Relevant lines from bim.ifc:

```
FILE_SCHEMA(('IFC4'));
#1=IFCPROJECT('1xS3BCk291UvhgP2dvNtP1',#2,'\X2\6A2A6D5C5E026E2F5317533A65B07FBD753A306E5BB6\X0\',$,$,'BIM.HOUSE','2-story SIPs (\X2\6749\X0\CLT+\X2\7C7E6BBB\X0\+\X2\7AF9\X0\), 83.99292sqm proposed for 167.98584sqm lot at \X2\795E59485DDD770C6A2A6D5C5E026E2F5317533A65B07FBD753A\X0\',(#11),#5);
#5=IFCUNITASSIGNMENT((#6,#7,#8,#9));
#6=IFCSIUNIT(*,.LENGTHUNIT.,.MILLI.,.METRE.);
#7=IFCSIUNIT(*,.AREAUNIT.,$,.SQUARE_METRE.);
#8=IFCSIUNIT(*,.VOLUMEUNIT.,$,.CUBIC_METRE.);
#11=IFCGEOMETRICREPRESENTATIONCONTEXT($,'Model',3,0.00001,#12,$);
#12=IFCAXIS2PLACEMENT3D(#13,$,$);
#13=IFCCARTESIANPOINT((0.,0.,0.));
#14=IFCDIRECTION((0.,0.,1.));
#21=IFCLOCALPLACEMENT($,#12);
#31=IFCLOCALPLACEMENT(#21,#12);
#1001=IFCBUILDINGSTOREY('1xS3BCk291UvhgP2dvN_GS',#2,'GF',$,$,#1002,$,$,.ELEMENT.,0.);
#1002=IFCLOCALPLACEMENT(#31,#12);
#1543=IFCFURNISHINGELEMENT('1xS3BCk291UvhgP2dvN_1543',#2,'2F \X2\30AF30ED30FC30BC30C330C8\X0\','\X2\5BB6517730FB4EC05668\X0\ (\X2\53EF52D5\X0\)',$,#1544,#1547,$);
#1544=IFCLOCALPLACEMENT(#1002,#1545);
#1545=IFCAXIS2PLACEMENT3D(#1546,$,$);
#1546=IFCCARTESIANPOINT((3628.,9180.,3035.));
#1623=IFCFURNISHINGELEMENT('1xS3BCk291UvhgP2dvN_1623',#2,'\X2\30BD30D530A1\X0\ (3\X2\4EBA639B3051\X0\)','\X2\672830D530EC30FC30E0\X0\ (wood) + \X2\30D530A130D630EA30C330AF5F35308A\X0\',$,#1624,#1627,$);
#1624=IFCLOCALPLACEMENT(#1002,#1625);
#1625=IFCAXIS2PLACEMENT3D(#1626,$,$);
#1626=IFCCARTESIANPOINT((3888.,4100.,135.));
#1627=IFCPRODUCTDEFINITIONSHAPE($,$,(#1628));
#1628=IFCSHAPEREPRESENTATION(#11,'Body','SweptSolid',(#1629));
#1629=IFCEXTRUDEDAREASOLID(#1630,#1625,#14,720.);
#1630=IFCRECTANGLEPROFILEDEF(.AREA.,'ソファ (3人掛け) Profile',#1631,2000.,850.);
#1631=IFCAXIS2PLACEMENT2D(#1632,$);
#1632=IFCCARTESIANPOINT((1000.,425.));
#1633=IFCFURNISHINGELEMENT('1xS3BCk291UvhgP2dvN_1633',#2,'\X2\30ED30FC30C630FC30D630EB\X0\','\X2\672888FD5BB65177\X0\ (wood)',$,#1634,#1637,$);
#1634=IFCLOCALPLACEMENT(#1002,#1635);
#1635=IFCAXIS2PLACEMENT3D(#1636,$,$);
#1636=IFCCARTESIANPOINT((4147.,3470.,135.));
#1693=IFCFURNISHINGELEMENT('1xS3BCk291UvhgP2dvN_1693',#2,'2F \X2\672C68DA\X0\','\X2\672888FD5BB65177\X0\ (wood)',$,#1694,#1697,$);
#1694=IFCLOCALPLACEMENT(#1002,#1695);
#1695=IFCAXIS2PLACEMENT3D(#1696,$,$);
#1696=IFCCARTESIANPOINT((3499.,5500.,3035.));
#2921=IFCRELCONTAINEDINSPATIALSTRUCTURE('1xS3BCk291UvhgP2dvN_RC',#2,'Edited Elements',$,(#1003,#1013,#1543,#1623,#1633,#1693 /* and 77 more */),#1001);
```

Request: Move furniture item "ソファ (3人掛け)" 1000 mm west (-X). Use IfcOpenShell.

```python
import ifcopenshell
import ifcopenshell.api.geometry
import ifcopenshell.util.placement
import ifcopenshell.util.unit

model = ifcopenshell.open("bim.ifc")
unit_scale = ifcopenshell.util.unit.calculate_unit_scale(model)

item = model.by_id(1623)
matrix = ifcopenshell.util.placement.get_local_placement(item.ObjectPlacement)
matrix[0, 3] -= 1 / unit_scale
ifcopenshell.api.geometry.edit_object_placement(model, product=item, matrix=matrix, is_si=False)

print(ifcopenshell.util.placement.get_local_placement(item.ObjectPlacement).round(3) + 0.0)

model.write("bim_rev.ifc")
```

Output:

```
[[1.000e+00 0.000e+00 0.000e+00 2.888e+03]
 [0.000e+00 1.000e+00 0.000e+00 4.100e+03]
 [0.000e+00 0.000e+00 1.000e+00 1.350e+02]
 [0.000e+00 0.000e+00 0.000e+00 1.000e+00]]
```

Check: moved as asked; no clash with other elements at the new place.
